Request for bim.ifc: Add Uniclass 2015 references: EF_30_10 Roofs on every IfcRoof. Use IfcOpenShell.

First a look at what the model holds.

```python
import ifcopenshell

model = ifcopenshell.open("bim.ifc")
print(model.schema)
print("classifications:", [c.Name for c in model.by_type("IfcClassification")])
for ifc_class in ("IfcDoor", "IfcRoof", "IfcStair", "IfcWall", "IfcWindow"):
    print(ifc_class, len(model.by_type(ifc_class)))
```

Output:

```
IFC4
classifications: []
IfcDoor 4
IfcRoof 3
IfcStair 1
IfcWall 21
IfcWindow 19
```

```python
import ifcopenshell
import ifcopenshell.api.classification

model = ifcopenshell.open("bim.ifc")

system = ifcopenshell.api.classification.add_classification(model, classification="Uniclass 2015")

codes = {
    "IfcRoof": ("EF_30_10", "Roofs"),
}
for ifc_class, (code, name) in codes.items():
    products = model.by_type(ifc_class)
    ifcopenshell.api.classification.add_reference(
        model, products=products, classification=system, identification=code, name=name
    )
    print(code, len(products))

model.write("bim-out.ifc")
```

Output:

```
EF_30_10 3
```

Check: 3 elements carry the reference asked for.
